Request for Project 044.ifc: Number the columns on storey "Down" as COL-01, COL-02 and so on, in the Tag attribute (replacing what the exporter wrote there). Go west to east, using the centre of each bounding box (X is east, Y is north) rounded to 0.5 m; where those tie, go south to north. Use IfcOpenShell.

First a look at what the model holds.

```python
import ifcopenshell
import ifcopenshell.util.element
import ifcopenshell.util.placement

model = ifcopenshell.open("Project 044.ifc")
print(model.schema)
storey = next(s for s in model.by_type("IfcBuildingStorey") if s.Name == "Down")
columns = [e for e in ifcopenshell.util.element.get_decomposition(storey) if e.is_a("IfcColumn")]
for e in sorted(columns, key=lambda e: e.id()):
    origin = ifcopenshell.util.placement.get_local_placement(e.ObjectPlacement)[:3, 3]
    print(e.id(), e.Tag, e.Name, origin.round(2) + 0.0, sep=" | ")
```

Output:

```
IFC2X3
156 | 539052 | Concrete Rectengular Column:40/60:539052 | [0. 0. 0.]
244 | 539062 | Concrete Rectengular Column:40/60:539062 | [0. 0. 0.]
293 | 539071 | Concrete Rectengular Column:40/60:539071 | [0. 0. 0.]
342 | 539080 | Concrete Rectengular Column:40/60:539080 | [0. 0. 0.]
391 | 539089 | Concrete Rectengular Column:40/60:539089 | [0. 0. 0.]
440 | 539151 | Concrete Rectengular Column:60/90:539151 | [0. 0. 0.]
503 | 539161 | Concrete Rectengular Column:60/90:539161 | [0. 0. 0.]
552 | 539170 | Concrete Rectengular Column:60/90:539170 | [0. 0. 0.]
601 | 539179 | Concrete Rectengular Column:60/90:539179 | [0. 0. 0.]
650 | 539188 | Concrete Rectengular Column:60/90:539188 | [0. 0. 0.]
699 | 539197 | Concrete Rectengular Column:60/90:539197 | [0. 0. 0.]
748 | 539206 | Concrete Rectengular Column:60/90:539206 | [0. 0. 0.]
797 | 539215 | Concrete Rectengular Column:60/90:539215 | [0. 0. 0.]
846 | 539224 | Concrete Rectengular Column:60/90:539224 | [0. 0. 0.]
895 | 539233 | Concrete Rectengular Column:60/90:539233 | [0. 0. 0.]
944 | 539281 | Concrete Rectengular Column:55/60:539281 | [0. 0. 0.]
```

```python
import ifcopenshell
import ifcopenshell.geom
import ifcopenshell.util.element
import ifcopenshell.util.shape

model = ifcopenshell.open("Project 044.ifc")
settings = ifcopenshell.geom.settings()
settings.set("use-world-coords", True)


def centre(element):
    shape = ifcopenshell.geom.create_shape(settings, element)
    return ifcopenshell.util.shape.get_bbox_centroid(shape.geometry)


storey = next(s for s in model.by_type("IfcBuildingStorey") if s.Name == "Down")
columns = [e for e in ifcopenshell.util.element.get_decomposition(storey) if e.is_a("IfcColumn")]

# Insertion points can sit at a corner or the storey origin, so sort by the geometry (in metres).
centres = {e: centre(e) for e in columns}
columns.sort(key=lambda e: (round(centres[e][0] / 0.5), centres[e][1]))

for i, e in enumerate(columns, start=1):
    number = f"COL-{i:02d}"
    e.Tag = number
    print(e.id(), number)

model.write("Project 044_updated.ifc")
```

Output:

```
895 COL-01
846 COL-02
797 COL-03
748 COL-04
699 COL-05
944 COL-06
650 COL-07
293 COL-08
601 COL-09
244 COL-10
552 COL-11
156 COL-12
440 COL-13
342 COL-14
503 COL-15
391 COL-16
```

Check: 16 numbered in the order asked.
